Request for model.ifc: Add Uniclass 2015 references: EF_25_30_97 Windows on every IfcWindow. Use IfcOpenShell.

First a look at what the model holds.

```python
import ifcopenshell

model = ifcopenshell.open("model.ifc")
print(model.schema)
print("classifications:", [c.Name for c in model.by_type("IfcClassification")])
for ifc_class in ("IfcDoor", "IfcRoof", "IfcStair", "IfcWall", "IfcWindow"):
    print(ifc_class, len(model.by_type(ifc_class)))
```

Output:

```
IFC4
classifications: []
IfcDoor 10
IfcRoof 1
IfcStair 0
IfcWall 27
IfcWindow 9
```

```python
import ifcopenshell
import ifcopenshell.api.classification

model = ifcopenshell.open("model.ifc")

system = ifcopenshell.api.classification.add_classification(model, classification="Uniclass 2015")

codes = {
    "IfcWindow": ("EF_25_30_97", "Windows"),
}
for ifc_class, (code, name) in codes.items():
    products = model.by_type(ifc_class)
    ifcopenshell.api.classification.add_reference(
        model, products=products, classification=system, identification=code, name=name
    )
    print(code, len(products))

model.write("model_rev.ifc")
```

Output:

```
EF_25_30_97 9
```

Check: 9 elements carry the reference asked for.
